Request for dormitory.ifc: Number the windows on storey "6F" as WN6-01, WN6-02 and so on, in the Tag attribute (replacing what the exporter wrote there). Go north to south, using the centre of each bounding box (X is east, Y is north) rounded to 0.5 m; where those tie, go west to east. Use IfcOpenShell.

First a look at what the model holds.

```python
import ifcopenshell
import ifcopenshell.util.element
import ifcopenshell.util.placement

model = ifcopenshell.open("dormitory.ifc")
print(model.schema)
storey = next(s for s in model.by_type("IfcBuildingStorey") if s.Name == "6F")
windows = [e for e in ifcopenshell.util.element.get_decomposition(storey) if e.is_a("IfcWindow")]
for e in sorted(windows, key=lambda e: e.id()):
    origin = ifcopenshell.util.placement.get_local_placement(e.ObjectPlacement)[:3, 3]
    print(e.id(), e.Tag, e.Name, origin.round(2) + 0.0, sep=" | ")
```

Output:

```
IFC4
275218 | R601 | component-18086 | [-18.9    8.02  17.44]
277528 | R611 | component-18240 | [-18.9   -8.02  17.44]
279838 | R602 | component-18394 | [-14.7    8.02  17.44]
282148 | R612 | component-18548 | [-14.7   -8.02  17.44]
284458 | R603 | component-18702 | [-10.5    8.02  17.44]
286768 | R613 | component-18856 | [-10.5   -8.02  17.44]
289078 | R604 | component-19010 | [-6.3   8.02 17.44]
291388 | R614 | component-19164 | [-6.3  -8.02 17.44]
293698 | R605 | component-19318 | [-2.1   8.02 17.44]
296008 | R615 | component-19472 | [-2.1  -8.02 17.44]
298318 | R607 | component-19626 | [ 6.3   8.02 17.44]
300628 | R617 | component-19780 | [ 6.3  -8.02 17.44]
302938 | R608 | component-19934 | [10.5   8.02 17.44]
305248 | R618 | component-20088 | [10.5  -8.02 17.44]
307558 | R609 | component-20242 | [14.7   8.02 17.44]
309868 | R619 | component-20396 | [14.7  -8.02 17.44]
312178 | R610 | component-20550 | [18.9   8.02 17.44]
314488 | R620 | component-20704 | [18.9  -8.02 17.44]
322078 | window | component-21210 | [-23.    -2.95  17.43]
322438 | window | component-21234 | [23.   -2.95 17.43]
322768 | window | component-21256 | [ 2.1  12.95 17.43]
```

```python
import ifcopenshell
import ifcopenshell.geom
import ifcopenshell.util.element
import ifcopenshell.util.shape

model = ifcopenshell.open("dormitory.ifc")
settings = ifcopenshell.geom.settings()
settings.set("use-world-coords", True)


def centre(element):
    shape = ifcopenshell.geom.create_shape(settings, element)
    return ifcopenshell.util.shape.get_bbox_centroid(shape.geometry)


storey = next(s for s in model.by_type("IfcBuildingStorey") if s.Name == "6F")
windows = [e for e in ifcopenshell.util.element.get_decomposition(storey) if e.is_a("IfcWindow")]

# Insertion points can sit at a corner or the storey origin, so sort by the geometry (in metres).
centres = {e: centre(e) for e in windows}
windows.sort(key=lambda e: (-round(centres[e][1] / 0.5), centres[e][0]))

for i, e in enumerate(windows, start=1):
    number = f"WN6-{i:02d}"
    e.Tag = number
    print(e.id(), number)

model.write("dormitory_rev.ifc")
```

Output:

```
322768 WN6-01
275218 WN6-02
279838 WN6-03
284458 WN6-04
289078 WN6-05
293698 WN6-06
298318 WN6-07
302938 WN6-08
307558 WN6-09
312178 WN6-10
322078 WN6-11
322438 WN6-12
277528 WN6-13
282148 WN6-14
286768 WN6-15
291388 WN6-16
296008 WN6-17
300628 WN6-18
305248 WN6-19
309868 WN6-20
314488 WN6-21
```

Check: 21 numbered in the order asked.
